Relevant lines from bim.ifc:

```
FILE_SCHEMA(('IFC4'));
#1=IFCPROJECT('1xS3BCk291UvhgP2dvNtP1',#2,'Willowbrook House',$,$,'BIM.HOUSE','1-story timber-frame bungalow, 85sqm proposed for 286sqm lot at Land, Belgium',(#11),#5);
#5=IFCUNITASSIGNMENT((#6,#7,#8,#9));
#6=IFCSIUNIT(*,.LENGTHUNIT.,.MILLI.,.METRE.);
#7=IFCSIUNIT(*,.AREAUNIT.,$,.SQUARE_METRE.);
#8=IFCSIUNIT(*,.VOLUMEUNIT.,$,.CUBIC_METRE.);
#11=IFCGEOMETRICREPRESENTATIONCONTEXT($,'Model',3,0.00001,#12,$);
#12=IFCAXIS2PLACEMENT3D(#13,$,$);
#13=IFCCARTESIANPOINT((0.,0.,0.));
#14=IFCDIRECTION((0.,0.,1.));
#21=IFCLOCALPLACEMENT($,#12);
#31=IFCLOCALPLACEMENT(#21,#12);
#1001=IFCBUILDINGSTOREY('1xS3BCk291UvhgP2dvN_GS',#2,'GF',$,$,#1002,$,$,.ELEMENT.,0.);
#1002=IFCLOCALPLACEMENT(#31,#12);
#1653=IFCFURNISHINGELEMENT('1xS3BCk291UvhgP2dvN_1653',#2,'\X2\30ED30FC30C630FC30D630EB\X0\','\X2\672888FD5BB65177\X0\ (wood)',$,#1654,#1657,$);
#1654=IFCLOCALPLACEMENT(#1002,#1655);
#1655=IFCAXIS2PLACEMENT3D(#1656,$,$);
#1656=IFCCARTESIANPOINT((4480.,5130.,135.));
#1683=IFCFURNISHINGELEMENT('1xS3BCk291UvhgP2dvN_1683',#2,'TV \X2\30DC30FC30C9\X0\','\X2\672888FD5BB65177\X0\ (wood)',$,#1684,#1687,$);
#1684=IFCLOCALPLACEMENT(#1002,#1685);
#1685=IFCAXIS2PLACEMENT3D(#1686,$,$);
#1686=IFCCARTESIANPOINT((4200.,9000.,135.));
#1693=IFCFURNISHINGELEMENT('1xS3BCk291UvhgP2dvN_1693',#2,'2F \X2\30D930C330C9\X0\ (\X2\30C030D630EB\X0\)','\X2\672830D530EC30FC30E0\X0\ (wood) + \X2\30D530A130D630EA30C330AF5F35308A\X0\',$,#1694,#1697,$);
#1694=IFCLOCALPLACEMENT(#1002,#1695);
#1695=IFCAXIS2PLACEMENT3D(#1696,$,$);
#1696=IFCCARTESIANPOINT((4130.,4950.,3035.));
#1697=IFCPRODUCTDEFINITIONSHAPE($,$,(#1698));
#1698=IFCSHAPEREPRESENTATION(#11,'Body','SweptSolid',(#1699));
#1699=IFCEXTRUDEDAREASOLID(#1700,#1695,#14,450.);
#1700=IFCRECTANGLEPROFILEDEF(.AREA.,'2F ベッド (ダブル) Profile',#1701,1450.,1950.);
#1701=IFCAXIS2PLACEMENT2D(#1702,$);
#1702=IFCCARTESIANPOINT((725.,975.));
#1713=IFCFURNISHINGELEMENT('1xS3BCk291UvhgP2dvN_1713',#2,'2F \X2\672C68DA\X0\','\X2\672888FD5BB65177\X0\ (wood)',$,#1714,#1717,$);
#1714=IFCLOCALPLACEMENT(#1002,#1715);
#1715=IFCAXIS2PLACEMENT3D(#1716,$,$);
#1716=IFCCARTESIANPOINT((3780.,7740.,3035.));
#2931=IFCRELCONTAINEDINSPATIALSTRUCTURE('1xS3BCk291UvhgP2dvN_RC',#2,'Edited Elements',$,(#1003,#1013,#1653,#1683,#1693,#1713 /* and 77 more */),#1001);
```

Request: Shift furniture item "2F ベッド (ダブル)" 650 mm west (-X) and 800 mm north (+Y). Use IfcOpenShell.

```python
import ifcopenshell
import ifcopenshell.api.geometry
import ifcopenshell.util.placement

model = ifcopenshell.open("bim.ifc")

item = model.by_guid("1xS3BCk291UvhgP2dvN_1693")
matrix = ifcopenshell.util.placement.get_local_placement(item.ObjectPlacement)
matrix[0, 3] -= 650.0
matrix[1, 3] += 800.0
ifcopenshell.api.geometry.edit_object_placement(model, product=item, matrix=matrix, is_si=False)

print(ifcopenshell.util.placement.get_local_placement(item.ObjectPlacement).round(3) + 0.0)

model.write("bim_edited.ifc")
```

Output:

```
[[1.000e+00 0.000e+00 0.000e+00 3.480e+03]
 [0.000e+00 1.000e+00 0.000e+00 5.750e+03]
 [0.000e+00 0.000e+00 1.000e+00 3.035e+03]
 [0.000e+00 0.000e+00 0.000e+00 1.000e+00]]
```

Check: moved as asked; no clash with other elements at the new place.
